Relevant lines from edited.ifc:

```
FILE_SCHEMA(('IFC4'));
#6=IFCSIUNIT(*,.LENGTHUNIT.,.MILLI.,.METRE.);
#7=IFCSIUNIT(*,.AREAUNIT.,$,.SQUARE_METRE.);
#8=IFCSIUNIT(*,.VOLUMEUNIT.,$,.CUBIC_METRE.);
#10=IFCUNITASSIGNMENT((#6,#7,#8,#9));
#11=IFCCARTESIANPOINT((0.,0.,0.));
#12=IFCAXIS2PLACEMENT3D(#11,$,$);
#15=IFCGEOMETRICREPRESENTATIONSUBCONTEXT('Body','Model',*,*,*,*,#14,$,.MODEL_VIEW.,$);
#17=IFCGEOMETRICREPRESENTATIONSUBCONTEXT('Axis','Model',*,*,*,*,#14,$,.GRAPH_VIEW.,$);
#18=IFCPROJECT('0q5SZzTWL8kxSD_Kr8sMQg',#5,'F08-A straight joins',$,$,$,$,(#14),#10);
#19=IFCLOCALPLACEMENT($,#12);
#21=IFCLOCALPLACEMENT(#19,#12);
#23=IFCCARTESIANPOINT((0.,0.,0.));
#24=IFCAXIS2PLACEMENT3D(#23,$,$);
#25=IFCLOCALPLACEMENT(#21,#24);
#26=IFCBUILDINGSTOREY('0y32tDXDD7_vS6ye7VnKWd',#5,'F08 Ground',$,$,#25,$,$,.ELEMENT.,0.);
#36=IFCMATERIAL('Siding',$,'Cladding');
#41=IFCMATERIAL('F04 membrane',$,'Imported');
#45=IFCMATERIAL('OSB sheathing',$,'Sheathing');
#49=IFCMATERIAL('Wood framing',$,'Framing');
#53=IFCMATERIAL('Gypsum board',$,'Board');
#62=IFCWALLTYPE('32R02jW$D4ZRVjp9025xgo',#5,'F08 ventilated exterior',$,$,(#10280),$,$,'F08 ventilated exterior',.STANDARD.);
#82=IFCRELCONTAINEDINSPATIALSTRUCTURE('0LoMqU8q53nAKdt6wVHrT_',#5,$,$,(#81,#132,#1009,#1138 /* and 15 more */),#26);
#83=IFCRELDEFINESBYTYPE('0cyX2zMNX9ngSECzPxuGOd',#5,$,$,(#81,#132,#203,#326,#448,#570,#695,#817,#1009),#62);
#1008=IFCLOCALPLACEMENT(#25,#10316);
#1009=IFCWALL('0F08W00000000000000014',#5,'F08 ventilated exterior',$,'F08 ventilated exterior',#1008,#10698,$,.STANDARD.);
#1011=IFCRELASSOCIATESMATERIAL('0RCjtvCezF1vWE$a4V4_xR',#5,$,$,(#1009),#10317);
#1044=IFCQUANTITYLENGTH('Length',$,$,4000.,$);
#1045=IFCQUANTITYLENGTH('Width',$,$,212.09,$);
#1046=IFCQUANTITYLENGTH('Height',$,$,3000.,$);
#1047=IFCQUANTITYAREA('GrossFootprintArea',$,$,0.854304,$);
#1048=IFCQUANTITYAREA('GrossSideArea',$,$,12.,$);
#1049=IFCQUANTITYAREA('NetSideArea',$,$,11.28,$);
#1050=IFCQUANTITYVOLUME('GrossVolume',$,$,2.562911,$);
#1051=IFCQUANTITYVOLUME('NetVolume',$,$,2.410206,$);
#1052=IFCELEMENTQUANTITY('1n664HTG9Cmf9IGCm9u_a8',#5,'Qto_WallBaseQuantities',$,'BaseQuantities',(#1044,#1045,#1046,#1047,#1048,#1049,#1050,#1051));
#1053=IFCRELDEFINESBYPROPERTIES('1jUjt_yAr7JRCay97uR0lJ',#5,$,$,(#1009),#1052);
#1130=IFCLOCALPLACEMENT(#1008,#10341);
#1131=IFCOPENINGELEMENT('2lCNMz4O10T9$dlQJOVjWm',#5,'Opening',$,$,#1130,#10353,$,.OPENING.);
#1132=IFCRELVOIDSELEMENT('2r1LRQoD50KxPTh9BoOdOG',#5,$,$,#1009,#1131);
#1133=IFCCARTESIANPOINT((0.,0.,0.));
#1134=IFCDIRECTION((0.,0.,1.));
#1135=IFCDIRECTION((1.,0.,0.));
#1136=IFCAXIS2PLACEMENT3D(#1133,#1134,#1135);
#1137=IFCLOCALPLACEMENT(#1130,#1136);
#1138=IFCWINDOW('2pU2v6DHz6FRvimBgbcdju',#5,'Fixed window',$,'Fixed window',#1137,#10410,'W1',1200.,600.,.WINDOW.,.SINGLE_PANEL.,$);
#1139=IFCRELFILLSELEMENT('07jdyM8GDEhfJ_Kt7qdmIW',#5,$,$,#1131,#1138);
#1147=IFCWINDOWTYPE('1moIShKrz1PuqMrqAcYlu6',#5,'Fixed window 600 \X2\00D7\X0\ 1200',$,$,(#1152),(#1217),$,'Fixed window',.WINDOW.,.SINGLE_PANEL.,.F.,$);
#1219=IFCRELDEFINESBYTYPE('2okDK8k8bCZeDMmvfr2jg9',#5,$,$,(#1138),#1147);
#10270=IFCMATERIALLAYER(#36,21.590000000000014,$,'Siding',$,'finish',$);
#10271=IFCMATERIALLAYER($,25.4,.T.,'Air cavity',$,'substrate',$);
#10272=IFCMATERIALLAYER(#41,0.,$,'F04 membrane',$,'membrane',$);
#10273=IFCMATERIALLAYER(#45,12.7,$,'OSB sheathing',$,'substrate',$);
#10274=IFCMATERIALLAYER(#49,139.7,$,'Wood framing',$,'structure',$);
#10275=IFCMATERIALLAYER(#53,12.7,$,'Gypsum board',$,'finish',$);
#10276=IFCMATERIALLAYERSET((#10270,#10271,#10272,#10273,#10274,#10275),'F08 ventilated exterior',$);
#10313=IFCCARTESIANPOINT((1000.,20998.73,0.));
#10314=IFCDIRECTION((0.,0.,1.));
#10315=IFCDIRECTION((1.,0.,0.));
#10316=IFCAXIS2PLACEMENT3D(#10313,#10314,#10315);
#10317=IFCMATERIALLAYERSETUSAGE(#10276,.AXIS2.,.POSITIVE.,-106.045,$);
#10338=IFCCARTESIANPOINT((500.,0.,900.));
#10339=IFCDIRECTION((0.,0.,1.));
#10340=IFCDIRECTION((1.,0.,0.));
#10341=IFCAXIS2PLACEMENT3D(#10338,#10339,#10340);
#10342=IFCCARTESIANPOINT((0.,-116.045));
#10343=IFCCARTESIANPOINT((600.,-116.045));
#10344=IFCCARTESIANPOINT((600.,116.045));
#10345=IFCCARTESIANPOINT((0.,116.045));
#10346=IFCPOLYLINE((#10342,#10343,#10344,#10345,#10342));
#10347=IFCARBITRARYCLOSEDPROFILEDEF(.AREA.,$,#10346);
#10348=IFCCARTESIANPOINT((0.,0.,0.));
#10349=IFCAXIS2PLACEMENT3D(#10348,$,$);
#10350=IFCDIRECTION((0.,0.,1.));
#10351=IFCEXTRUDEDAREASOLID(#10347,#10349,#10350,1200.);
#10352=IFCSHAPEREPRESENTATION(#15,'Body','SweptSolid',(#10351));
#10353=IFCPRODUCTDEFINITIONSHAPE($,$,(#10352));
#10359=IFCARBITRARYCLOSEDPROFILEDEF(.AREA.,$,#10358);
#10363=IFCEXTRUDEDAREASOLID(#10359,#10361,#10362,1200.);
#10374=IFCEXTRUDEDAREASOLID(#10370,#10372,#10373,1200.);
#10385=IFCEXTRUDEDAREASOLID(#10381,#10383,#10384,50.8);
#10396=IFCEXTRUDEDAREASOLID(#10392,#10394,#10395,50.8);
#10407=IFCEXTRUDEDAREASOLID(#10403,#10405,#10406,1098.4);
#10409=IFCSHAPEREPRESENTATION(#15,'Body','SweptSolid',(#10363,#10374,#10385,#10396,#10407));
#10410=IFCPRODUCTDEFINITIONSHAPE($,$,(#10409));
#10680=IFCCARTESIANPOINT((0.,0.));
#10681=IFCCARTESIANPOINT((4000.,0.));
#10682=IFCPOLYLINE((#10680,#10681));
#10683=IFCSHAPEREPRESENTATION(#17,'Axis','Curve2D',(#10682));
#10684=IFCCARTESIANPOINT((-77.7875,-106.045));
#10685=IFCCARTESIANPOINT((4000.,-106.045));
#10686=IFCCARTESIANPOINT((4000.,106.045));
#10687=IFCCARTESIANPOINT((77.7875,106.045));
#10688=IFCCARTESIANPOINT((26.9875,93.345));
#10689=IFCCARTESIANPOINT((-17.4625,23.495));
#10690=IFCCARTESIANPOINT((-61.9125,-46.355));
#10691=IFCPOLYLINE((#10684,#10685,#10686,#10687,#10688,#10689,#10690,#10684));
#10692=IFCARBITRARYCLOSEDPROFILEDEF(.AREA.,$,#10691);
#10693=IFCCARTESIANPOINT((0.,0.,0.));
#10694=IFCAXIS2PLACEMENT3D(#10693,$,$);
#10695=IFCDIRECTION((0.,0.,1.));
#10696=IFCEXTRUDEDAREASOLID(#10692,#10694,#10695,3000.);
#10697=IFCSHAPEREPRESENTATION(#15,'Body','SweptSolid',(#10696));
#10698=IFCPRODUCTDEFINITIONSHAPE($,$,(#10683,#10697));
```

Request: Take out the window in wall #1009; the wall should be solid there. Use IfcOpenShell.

```python
import ifcopenshell
import ifcopenshell.api.feature
import ifcopenshell.api.pset
import ifcopenshell.api.root
import ifcopenshell.geom
import ifcopenshell.util.element
import ifcopenshell.util.shape
import ifcopenshell.util.unit

model = ifcopenshell.open("edited.ifc")
area_scale = ifcopenshell.util.unit.calculate_unit_scale(model, "AREAUNIT")
volume_scale = ifcopenshell.util.unit.calculate_unit_scale(model, "VOLUMEUNIT")
settings = ifcopenshell.geom.settings()


def volume(element):
    """Net volume in cubic metres, openings subtracted."""
    shape = ifcopenshell.geom.create_shape(settings, element)
    return ifcopenshell.util.shape.get_volume(shape.geometry)


window = model.by_guid("2pU2v6DHz6FRvimBgbcdju")
opening = window.FillsVoids[0].RelatingOpeningElement
wall = opening.VoidsElements[0].RelatingBuildingElement
before = volume(wall)

ifcopenshell.api.root.remove_product(model, product=window)
ifcopenshell.api.feature.remove_feature(model, feature=opening)

after = volume(wall)
thickness = 0.2121  # wall thickness in metres

# Update the wall's stored quantities.
qto = model.by_id(ifcopenshell.util.element.get_pset(wall, "Qto_WallBaseQuantities", should_inherit=False)["id"])
ifcopenshell.api.pset.edit_qto(model, qto=qto, properties={
    "NetSideArea": after / thickness / area_scale,
    "NetVolume": after / volume_scale,
})

print(f"wall volume {before:.3f} -> {after:.3f} m3")

model.write("edited-out.ifc")
```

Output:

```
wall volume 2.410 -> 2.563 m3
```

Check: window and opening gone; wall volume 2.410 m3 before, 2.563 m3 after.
